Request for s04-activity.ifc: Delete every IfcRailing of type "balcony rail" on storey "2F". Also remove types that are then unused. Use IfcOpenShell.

First a look at what the model holds.

```python
import ifcopenshell
import ifcopenshell.util.element

model = ifcopenshell.open("s04-activity.ifc")
print(model.schema)
storey = next(s for s in model.by_type("IfcBuildingStorey") if s.Name == "2F")
railings = [e for e in ifcopenshell.util.element.get_decomposition(storey) if e.is_a("IfcRailing")]
seen = {}
for e in railings:
    element_type = ifcopenshell.util.element.get_type(e)
    name = element_type.Name if element_type not in (None, e) else None
    seen[name] = seen.get(name, 0) + 1
for name, count in sorted(seen.items(), key=str):
    print(count, "x", name)
```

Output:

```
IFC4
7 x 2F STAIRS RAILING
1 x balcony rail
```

```python
import ifcopenshell
import ifcopenshell.api.root
import ifcopenshell.util.element

model = ifcopenshell.open("s04-activity.ifc")

storey = next(s for s in model.by_type("IfcBuildingStorey") if s.Name == "2F")
railings = [e for e in ifcopenshell.util.element.get_decomposition(storey) if e.is_a("IfcRailing")]
targets = [e for e in railings if (t := ifcopenshell.util.element.get_type(e)) not in (None, e) and t.Name == "balcony rail"]
types = {ifcopenshell.util.element.get_type(e) for e in targets} - {None, *targets}

for e in targets:
    ifcopenshell.api.root.remove_product(model, product=e)
print(len(targets), "removed")

unused = [t for t in types if not ifcopenshell.util.element.get_types(t)]
for t in unused:
    ifcopenshell.api.root.remove_product(model, product=t)
print(len(unused), "unused types removed")

model.write("s04-activity_rev.ifc")
```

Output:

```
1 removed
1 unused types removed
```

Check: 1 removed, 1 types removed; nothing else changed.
